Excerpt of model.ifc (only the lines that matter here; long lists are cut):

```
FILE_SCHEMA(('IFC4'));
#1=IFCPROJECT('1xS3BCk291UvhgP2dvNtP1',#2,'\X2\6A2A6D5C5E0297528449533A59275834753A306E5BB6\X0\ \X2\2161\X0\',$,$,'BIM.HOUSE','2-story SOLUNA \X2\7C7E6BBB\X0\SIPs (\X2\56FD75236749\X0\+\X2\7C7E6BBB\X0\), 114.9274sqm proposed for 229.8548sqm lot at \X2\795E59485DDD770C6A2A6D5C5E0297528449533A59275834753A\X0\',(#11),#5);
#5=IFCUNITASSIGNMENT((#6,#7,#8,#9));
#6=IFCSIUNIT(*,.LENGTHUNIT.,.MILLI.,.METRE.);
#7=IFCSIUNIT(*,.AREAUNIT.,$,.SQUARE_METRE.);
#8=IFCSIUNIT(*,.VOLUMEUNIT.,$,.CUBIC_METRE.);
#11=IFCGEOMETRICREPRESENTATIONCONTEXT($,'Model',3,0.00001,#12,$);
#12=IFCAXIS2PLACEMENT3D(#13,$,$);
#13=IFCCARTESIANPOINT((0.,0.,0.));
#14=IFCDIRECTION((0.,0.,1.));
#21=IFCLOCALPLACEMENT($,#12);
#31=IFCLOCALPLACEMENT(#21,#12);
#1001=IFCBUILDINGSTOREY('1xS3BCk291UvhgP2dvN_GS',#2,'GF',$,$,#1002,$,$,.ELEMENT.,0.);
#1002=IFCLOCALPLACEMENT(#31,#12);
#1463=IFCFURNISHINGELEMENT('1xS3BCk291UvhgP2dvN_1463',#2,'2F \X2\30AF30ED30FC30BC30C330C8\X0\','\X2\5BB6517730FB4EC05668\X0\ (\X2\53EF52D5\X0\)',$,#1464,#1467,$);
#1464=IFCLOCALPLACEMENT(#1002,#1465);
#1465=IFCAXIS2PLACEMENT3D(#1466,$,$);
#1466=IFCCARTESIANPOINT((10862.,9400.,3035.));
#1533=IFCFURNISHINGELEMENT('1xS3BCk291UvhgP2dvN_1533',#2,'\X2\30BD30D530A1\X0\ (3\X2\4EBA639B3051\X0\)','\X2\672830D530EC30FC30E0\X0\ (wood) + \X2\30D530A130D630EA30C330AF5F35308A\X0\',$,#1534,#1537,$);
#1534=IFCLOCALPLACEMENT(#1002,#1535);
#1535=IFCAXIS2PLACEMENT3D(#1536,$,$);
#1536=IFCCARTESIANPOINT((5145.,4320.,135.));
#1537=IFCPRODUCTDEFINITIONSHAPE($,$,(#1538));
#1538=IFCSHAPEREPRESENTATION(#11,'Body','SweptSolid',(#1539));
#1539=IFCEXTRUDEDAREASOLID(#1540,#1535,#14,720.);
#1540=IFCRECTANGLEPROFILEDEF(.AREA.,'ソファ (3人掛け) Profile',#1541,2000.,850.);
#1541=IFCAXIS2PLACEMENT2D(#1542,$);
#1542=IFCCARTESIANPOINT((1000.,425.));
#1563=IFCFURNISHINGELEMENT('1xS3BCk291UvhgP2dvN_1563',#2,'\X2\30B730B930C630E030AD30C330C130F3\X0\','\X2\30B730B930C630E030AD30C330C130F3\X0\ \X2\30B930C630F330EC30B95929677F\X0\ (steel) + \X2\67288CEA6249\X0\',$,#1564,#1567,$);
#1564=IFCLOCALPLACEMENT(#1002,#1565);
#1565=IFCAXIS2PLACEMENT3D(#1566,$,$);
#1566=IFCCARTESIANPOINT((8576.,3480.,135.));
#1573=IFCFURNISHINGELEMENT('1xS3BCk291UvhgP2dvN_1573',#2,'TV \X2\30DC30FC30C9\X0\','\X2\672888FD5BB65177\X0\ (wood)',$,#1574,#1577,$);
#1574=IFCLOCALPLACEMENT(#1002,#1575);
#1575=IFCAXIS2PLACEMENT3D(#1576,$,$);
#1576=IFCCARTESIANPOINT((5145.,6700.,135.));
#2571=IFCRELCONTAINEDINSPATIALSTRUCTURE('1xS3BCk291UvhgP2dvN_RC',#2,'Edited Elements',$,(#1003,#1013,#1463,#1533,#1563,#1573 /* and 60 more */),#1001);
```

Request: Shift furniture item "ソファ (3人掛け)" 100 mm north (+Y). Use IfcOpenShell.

```python
import ifcopenshell
import ifcopenshell.api.geometry
import ifcopenshell.util.placement
import ifcopenshell.util.unit

model = ifcopenshell.open("model.ifc")
unit_scale = ifcopenshell.util.unit.calculate_unit_scale(model)

item = model.by_guid("1xS3BCk291UvhgP2dvN_1533")
matrix = ifcopenshell.util.placement.get_local_placement(item.ObjectPlacement)
matrix[1, 3] += 0.1 / unit_scale
ifcopenshell.api.geometry.edit_object_placement(model, product=item, matrix=matrix, is_si=False)

print(ifcopenshell.util.placement.get_local_placement(item.ObjectPlacement).round(3) + 0.0)

model.write("model_v2.ifc")
```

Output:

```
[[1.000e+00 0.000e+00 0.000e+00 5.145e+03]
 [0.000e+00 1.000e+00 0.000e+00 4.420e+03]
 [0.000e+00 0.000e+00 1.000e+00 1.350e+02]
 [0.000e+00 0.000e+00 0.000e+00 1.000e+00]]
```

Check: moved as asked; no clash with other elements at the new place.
